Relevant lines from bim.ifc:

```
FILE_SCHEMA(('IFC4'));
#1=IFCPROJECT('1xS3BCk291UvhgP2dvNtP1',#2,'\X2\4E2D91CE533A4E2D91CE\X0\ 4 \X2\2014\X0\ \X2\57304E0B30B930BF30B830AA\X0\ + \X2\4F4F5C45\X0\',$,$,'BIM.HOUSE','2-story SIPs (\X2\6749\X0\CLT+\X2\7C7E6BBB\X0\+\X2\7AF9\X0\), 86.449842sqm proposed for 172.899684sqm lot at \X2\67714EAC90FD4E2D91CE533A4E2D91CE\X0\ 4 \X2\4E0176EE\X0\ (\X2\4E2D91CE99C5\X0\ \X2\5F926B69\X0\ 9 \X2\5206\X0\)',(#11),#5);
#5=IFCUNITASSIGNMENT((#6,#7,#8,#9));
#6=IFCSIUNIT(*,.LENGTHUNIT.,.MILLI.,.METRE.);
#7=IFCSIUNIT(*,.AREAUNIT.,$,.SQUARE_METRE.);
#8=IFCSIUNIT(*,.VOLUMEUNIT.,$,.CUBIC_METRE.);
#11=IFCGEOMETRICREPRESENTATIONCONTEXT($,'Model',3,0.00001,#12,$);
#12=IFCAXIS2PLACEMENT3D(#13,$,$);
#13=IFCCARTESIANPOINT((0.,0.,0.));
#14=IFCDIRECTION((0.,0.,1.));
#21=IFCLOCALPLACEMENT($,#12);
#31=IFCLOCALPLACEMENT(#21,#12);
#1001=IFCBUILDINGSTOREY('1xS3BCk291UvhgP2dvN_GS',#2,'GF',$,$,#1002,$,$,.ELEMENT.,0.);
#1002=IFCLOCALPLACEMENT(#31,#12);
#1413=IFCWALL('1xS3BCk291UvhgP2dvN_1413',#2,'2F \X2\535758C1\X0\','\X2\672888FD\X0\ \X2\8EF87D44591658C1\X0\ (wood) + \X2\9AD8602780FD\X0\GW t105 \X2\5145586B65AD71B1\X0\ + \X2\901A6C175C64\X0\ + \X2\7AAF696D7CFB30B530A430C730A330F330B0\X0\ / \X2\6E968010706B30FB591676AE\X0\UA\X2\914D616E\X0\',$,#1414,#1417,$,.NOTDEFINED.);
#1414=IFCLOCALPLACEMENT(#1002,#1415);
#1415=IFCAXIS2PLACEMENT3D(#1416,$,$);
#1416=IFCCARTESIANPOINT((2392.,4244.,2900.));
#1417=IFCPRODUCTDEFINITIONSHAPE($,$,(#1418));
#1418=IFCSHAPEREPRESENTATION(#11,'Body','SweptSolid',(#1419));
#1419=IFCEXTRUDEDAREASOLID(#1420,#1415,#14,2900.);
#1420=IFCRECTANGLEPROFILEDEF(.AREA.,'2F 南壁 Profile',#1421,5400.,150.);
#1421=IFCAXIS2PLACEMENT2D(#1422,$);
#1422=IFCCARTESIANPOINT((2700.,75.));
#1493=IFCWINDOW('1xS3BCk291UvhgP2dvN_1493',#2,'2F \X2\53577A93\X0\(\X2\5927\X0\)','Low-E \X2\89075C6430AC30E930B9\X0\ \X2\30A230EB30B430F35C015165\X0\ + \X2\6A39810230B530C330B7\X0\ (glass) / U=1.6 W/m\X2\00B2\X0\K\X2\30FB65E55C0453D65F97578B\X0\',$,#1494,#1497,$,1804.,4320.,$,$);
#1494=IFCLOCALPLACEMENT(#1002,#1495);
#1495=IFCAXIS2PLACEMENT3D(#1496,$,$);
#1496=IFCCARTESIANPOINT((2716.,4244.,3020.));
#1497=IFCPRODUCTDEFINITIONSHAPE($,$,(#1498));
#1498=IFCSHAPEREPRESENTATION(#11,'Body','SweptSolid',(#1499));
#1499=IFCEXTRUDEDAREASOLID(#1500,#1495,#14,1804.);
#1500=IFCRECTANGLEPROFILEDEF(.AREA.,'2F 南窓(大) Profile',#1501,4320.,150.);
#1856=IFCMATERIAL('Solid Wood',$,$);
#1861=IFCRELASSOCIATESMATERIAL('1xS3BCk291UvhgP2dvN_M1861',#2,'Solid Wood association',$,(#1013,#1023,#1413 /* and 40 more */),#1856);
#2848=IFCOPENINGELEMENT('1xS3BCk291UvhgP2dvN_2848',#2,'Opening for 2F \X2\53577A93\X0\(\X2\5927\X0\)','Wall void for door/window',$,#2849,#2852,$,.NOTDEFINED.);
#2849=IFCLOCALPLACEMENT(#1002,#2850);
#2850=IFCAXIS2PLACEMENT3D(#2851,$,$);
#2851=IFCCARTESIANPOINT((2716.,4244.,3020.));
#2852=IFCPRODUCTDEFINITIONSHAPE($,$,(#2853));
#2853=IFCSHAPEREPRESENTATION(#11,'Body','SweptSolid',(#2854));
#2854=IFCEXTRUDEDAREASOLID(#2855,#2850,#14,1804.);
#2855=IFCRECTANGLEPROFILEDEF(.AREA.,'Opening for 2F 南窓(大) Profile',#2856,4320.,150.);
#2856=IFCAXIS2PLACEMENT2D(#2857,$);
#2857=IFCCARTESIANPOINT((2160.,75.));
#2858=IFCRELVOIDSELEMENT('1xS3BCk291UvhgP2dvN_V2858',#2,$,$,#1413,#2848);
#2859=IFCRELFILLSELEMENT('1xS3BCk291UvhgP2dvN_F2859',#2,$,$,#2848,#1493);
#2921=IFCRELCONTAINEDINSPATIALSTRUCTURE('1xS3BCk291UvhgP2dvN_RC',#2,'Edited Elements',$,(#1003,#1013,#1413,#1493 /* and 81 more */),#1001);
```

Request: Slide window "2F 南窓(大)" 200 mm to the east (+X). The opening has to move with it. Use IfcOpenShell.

```python
import ifcopenshell
import ifcopenshell.api.geometry
import ifcopenshell.util.placement
import ifcopenshell.util.unit

model = ifcopenshell.open("bim.ifc")
unit_scale = ifcopenshell.util.unit.calculate_unit_scale(model)

window = model.by_id(1493)
opening = window.FillsVoids[0].RelatingOpeningElement
wall = opening.VoidsElements[0].RelatingBuildingElement

wall_matrix = ifcopenshell.util.placement.get_local_placement(wall.ObjectPlacement)
shift = wall_matrix[:3, 0] * 0.2 / unit_scale
before = ifcopenshell.util.placement.get_local_placement(window.ObjectPlacement)[:3, 3].copy()

# The window is not placed relative to its opening, so move both.
for product in (opening, window):
    matrix = ifcopenshell.util.placement.get_local_placement(product.ObjectPlacement)
    matrix[:3, 3] += shift
    ifcopenshell.api.geometry.edit_object_placement(model, product=product, matrix=matrix, is_si=False)

after = ifcopenshell.util.placement.get_local_placement(window.ObjectPlacement)[:3, 3]
print("window moved by", (after - before).round(3) + 0.0)

model.write("bim_v2.ifc")
```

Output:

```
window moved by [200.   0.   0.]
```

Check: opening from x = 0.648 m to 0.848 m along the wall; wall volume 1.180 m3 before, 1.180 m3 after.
